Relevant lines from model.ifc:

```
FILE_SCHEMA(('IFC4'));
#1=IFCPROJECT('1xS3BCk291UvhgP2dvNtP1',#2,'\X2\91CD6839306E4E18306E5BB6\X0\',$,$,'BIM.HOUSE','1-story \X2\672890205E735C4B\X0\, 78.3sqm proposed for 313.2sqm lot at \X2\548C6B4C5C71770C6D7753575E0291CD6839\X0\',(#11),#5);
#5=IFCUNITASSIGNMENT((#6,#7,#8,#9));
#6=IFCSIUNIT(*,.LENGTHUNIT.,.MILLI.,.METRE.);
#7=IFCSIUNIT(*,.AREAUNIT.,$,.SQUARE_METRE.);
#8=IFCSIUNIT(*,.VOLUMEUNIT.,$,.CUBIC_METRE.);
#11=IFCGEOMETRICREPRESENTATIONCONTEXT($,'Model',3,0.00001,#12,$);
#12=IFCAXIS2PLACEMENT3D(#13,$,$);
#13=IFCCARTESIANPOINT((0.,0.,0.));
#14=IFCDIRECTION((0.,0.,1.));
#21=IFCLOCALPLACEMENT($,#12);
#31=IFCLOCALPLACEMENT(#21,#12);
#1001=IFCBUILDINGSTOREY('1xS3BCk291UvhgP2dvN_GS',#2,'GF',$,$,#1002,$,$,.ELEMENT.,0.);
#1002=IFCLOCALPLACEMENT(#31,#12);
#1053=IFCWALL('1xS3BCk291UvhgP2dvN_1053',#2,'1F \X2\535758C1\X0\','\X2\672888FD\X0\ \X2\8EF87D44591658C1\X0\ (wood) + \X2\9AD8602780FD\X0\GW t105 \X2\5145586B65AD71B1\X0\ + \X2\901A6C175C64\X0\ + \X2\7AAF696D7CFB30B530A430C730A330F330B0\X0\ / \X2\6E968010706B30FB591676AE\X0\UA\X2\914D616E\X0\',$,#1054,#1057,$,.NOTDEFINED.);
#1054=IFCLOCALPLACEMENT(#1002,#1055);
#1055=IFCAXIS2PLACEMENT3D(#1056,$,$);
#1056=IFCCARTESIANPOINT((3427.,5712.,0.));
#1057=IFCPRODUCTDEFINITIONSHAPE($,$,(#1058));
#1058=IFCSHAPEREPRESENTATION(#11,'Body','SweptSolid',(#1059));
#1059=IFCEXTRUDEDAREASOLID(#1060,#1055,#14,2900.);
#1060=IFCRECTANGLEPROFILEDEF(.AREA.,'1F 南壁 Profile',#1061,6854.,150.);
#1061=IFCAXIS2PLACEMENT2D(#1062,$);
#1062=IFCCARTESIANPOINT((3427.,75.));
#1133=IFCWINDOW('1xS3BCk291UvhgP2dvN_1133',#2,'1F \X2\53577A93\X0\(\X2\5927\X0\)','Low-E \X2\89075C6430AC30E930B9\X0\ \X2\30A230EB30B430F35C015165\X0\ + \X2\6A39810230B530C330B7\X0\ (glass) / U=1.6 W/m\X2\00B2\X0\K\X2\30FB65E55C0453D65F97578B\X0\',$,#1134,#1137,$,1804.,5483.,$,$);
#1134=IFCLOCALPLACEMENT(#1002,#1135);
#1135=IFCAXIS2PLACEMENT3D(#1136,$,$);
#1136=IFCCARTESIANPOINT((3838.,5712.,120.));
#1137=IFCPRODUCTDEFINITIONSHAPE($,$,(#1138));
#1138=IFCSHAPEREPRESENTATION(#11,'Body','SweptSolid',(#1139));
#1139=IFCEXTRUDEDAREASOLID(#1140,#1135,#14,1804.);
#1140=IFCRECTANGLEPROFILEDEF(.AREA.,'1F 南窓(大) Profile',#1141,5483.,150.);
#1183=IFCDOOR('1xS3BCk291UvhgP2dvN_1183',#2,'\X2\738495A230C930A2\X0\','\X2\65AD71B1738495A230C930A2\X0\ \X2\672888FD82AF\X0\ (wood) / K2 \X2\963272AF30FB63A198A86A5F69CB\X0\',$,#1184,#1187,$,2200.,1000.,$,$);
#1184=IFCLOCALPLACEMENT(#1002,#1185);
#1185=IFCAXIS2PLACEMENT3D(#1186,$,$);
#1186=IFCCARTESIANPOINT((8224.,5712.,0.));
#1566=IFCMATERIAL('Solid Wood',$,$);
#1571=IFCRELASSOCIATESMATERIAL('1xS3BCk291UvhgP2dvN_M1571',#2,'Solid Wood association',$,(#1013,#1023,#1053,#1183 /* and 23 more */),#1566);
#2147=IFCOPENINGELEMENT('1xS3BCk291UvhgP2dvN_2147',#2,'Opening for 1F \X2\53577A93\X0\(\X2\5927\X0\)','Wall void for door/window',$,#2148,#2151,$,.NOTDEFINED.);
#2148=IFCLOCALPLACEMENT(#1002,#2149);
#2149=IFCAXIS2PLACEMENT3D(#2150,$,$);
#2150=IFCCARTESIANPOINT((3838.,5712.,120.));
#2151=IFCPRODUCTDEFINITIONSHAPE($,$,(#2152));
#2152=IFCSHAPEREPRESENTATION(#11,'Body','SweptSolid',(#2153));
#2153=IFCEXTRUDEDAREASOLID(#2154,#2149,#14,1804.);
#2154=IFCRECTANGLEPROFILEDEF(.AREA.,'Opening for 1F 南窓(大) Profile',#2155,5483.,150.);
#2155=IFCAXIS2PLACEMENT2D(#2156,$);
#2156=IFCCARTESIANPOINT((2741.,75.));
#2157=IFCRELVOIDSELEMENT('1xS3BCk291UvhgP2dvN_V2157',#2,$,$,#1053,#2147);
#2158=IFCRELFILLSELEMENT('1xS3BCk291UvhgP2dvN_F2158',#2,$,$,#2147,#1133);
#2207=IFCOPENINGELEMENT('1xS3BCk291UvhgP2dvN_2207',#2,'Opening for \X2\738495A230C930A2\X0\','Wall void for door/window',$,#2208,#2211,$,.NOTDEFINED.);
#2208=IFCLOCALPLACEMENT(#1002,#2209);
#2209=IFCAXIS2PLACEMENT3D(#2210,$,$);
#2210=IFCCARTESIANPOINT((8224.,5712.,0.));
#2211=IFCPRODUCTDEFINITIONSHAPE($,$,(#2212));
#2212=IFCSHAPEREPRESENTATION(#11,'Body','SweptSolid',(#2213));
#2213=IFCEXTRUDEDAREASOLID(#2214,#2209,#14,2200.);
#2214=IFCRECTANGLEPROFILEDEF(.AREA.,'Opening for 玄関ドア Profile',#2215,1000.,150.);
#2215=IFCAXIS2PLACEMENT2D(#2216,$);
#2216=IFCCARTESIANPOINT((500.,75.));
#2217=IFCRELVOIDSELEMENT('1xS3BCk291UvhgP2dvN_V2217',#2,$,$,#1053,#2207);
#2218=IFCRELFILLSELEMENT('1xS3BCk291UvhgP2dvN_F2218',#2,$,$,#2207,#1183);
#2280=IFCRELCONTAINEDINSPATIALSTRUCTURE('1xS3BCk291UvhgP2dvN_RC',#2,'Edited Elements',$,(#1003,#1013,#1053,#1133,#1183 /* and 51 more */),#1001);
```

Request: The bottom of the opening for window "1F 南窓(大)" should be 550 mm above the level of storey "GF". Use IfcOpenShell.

```python
import numpy as np
import ifcopenshell
import ifcopenshell.api.geometry
import ifcopenshell.geom
import ifcopenshell.util.element
import ifcopenshell.util.placement
import ifcopenshell.util.shape
import ifcopenshell.util.unit

model = ifcopenshell.open("model.ifc")
unit_scale = ifcopenshell.util.unit.calculate_unit_scale(model)

window = model.by_guid("1xS3BCk291UvhgP2dvN_1133")
opening = window.FillsVoids[0].RelatingOpeningElement
storey = ifcopenshell.util.element.get_container(window, ifc_class="IfcBuildingStorey")
level = ifcopenshell.util.placement.get_local_placement(storey.ObjectPlacement)[2, 3]

# The opening's origin need not be at the sill, so measure its lowest point.
shape = ifcopenshell.geom.create_shape(ifcopenshell.geom.settings(), opening)
bottom = ifcopenshell.util.shape.get_shape_bottom_elevation(shape, shape.geometry) / unit_scale
dz = level + 0.55 / unit_scale - bottom

shift = np.array([0.0, 0.0, dz])
# The window is not placed relative to its opening, so move both.
for product in (opening, window):
    matrix = ifcopenshell.util.placement.get_local_placement(product.ObjectPlacement)
    matrix[:3, 3] += shift
    ifcopenshell.api.geometry.edit_object_placement(model, product=product, matrix=matrix, is_si=False)

print(f"moved by {dz * unit_scale:+.3f} m")

model.write("model_rev.ifc")
```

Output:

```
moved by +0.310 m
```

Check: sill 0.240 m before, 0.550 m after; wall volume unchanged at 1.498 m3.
